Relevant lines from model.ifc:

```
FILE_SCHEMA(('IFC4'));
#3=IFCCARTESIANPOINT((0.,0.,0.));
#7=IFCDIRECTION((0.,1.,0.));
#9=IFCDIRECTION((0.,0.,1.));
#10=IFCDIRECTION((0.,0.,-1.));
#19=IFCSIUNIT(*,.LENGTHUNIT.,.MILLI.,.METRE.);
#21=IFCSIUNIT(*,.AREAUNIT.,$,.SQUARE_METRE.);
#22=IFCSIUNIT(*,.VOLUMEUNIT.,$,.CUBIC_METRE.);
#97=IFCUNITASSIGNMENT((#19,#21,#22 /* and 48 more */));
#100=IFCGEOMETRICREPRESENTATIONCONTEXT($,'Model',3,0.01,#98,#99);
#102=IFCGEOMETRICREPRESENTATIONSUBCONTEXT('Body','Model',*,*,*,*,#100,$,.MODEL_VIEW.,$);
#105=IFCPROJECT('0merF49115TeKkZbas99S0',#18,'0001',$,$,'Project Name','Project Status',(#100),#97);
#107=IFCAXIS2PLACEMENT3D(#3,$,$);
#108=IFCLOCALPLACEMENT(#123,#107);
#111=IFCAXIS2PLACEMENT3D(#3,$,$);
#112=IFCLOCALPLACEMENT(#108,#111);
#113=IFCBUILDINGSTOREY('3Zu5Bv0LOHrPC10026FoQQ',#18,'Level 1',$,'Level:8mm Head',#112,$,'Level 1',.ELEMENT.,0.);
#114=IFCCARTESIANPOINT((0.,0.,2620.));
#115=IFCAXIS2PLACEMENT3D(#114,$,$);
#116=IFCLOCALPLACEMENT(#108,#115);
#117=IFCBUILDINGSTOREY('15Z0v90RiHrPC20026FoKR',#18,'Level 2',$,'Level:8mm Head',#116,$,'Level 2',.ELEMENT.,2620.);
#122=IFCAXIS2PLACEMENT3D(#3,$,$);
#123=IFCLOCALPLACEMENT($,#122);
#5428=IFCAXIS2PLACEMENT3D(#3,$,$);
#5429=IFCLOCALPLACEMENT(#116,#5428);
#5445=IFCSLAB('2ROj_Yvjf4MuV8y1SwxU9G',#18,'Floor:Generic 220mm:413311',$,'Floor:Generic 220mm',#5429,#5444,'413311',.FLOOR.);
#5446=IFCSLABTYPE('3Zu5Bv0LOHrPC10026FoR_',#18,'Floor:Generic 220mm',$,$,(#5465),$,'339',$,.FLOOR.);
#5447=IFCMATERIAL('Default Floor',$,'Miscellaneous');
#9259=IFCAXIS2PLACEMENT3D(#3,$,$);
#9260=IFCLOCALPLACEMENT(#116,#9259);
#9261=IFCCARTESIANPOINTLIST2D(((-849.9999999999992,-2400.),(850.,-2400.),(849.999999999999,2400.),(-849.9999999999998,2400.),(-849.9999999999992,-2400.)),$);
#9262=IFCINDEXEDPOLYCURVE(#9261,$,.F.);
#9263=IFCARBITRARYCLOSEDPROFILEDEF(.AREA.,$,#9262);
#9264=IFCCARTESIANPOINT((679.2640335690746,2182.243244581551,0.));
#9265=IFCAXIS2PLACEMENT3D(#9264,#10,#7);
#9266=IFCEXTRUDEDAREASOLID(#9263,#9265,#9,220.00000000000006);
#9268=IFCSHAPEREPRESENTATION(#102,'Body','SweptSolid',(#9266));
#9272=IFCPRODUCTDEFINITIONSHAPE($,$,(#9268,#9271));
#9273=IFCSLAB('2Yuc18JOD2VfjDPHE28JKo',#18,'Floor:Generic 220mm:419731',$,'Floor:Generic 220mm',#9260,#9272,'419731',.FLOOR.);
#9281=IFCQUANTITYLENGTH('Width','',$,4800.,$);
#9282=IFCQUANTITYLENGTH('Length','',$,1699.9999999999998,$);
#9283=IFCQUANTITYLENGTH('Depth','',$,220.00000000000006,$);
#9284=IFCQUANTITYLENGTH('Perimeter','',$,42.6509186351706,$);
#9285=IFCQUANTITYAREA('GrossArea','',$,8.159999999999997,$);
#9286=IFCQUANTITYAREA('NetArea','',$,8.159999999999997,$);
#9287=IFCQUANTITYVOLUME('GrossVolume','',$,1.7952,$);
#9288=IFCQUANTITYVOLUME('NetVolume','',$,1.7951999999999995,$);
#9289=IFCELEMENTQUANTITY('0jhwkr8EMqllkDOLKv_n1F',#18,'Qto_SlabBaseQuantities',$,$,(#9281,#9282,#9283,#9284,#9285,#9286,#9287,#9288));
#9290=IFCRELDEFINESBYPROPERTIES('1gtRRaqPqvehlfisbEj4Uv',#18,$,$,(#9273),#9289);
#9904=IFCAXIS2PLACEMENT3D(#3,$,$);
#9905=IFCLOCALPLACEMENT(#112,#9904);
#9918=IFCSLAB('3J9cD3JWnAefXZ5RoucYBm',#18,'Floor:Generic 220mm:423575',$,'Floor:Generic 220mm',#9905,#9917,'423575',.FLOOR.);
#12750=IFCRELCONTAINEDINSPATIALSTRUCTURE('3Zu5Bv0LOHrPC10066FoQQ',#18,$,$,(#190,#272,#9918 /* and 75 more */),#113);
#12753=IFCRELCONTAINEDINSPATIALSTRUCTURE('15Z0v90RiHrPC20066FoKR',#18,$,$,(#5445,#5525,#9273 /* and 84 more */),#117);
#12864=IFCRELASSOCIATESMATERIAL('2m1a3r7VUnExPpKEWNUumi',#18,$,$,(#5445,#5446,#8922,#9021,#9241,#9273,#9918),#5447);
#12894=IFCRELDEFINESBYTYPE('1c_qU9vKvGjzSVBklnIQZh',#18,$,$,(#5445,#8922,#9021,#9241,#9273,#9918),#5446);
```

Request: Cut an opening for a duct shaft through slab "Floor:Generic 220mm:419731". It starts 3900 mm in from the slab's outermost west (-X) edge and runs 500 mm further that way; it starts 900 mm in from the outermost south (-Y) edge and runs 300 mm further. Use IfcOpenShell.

```python
import numpy as np
import ifcopenshell
import ifcopenshell.api.feature
import ifcopenshell.api.geometry
import ifcopenshell.api.pset
import ifcopenshell.api.root
import ifcopenshell.geom
import ifcopenshell.util.element
import ifcopenshell.util.placement
import ifcopenshell.util.representation
import ifcopenshell.util.shape
import ifcopenshell.util.unit

model = ifcopenshell.open("model.ifc")
unit_scale = ifcopenshell.util.unit.calculate_unit_scale(model)
area_scale = ifcopenshell.util.unit.calculate_unit_scale(model, "AREAUNIT")
volume_scale = ifcopenshell.util.unit.calculate_unit_scale(model, "VOLUMEUNIT")
settings = ifcopenshell.geom.settings()


def volume(element):
    """Net volume in cubic metres, openings subtracted."""
    shape = ifcopenshell.geom.create_shape(settings, element)
    return ifcopenshell.util.shape.get_volume(shape.geometry)


slab = model.by_guid("2Yuc18JOD2VfjDPHE28JKo")
before = volume(slab)

# Extent in the slab's own axes, in metres. The edges named are its -X and -Y sides.
slab_shape = ifcopenshell.geom.create_shape(settings, slab)
vertices = ifcopenshell.util.shape.get_vertices(slab_shape.geometry)
x_min, y_min, bottom = vertices.min(axis=0)
top = vertices[:, 2].max()

opening = ifcopenshell.api.root.create_entity(model, ifc_class="IfcOpeningElement", name="Duct shaft opening", predefined_type="OPENING")
context = ifcopenshell.util.representation.get_context(model, "Model", "Body", "MODEL_VIEW")
width, depth = 0.5, 0.3
outline = [(0.0, 0.0), (width, 0.0), (width, depth), (0.0, depth), (0.0, 0.0)]
# Overshoot both faces by 50 mm so the cut is clean.
shape = ifcopenshell.api.geometry.add_slab_representation(
    model, context=context, depth=top - bottom + 0.1, polyline=outline
)
ifcopenshell.api.geometry.assign_representation(model, product=opening, representation=shape)

matrix = ifcopenshell.util.placement.get_local_placement(slab.ObjectPlacement)
matrix[:, 3] = matrix @ np.append(np.array([x_min + 3.9, y_min + 0.9, bottom - 0.05]) / unit_scale, 1.0)
ifcopenshell.api.geometry.edit_object_placement(model, product=opening, matrix=matrix, is_si=False)
ifcopenshell.api.feature.add_feature(model, feature=opening, element=slab)

after = volume(slab)

# Update the slab's stored quantities.
qto = model.by_id(ifcopenshell.util.element.get_pset(slab, "Qto_SlabBaseQuantities", should_inherit=False)["id"])
ifcopenshell.api.pset.edit_qto(model, qto=qto, properties={
    "NetArea": after / (top - bottom) / area_scale,
    "NetVolume": after / volume_scale,
})

print(f"slab volume {before:.3f} -> {after:.3f} m3")

model.write("model_v2.ifc")
```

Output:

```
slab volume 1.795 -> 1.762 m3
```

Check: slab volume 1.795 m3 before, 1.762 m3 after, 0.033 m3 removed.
